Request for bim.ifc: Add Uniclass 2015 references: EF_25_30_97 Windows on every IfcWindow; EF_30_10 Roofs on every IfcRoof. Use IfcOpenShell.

First a look at what the model holds.

```python
import ifcopenshell

model = ifcopenshell.open("bim.ifc")
print(model.schema)
print("classifications:", [c.Name for c in model.by_type("IfcClassification")])
for ifc_class in ("IfcDoor", "IfcRoof", "IfcStair", "IfcWall", "IfcWindow"):
    print(ifc_class, len(model.by_type(ifc_class)))
```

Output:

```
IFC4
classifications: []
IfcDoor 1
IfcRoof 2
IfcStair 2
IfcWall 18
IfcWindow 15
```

```python
import ifcopenshell
import ifcopenshell.api.classification

model = ifcopenshell.open("bim.ifc")

system = ifcopenshell.api.classification.add_classification(model, classification="Uniclass 2015")

codes = {
    "IfcWindow": ("EF_25_30_97", "Windows"),
    "IfcRoof": ("EF_30_10", "Roofs"),
}
for ifc_class, (code, name) in codes.items():
    products = model.by_type(ifc_class)
    ifcopenshell.api.classification.add_reference(
        model, products=products, classification=system, identification=code, name=name
    )
    print(code, len(products))

model.write("bim-out.ifc")
```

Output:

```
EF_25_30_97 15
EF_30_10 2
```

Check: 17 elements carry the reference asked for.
